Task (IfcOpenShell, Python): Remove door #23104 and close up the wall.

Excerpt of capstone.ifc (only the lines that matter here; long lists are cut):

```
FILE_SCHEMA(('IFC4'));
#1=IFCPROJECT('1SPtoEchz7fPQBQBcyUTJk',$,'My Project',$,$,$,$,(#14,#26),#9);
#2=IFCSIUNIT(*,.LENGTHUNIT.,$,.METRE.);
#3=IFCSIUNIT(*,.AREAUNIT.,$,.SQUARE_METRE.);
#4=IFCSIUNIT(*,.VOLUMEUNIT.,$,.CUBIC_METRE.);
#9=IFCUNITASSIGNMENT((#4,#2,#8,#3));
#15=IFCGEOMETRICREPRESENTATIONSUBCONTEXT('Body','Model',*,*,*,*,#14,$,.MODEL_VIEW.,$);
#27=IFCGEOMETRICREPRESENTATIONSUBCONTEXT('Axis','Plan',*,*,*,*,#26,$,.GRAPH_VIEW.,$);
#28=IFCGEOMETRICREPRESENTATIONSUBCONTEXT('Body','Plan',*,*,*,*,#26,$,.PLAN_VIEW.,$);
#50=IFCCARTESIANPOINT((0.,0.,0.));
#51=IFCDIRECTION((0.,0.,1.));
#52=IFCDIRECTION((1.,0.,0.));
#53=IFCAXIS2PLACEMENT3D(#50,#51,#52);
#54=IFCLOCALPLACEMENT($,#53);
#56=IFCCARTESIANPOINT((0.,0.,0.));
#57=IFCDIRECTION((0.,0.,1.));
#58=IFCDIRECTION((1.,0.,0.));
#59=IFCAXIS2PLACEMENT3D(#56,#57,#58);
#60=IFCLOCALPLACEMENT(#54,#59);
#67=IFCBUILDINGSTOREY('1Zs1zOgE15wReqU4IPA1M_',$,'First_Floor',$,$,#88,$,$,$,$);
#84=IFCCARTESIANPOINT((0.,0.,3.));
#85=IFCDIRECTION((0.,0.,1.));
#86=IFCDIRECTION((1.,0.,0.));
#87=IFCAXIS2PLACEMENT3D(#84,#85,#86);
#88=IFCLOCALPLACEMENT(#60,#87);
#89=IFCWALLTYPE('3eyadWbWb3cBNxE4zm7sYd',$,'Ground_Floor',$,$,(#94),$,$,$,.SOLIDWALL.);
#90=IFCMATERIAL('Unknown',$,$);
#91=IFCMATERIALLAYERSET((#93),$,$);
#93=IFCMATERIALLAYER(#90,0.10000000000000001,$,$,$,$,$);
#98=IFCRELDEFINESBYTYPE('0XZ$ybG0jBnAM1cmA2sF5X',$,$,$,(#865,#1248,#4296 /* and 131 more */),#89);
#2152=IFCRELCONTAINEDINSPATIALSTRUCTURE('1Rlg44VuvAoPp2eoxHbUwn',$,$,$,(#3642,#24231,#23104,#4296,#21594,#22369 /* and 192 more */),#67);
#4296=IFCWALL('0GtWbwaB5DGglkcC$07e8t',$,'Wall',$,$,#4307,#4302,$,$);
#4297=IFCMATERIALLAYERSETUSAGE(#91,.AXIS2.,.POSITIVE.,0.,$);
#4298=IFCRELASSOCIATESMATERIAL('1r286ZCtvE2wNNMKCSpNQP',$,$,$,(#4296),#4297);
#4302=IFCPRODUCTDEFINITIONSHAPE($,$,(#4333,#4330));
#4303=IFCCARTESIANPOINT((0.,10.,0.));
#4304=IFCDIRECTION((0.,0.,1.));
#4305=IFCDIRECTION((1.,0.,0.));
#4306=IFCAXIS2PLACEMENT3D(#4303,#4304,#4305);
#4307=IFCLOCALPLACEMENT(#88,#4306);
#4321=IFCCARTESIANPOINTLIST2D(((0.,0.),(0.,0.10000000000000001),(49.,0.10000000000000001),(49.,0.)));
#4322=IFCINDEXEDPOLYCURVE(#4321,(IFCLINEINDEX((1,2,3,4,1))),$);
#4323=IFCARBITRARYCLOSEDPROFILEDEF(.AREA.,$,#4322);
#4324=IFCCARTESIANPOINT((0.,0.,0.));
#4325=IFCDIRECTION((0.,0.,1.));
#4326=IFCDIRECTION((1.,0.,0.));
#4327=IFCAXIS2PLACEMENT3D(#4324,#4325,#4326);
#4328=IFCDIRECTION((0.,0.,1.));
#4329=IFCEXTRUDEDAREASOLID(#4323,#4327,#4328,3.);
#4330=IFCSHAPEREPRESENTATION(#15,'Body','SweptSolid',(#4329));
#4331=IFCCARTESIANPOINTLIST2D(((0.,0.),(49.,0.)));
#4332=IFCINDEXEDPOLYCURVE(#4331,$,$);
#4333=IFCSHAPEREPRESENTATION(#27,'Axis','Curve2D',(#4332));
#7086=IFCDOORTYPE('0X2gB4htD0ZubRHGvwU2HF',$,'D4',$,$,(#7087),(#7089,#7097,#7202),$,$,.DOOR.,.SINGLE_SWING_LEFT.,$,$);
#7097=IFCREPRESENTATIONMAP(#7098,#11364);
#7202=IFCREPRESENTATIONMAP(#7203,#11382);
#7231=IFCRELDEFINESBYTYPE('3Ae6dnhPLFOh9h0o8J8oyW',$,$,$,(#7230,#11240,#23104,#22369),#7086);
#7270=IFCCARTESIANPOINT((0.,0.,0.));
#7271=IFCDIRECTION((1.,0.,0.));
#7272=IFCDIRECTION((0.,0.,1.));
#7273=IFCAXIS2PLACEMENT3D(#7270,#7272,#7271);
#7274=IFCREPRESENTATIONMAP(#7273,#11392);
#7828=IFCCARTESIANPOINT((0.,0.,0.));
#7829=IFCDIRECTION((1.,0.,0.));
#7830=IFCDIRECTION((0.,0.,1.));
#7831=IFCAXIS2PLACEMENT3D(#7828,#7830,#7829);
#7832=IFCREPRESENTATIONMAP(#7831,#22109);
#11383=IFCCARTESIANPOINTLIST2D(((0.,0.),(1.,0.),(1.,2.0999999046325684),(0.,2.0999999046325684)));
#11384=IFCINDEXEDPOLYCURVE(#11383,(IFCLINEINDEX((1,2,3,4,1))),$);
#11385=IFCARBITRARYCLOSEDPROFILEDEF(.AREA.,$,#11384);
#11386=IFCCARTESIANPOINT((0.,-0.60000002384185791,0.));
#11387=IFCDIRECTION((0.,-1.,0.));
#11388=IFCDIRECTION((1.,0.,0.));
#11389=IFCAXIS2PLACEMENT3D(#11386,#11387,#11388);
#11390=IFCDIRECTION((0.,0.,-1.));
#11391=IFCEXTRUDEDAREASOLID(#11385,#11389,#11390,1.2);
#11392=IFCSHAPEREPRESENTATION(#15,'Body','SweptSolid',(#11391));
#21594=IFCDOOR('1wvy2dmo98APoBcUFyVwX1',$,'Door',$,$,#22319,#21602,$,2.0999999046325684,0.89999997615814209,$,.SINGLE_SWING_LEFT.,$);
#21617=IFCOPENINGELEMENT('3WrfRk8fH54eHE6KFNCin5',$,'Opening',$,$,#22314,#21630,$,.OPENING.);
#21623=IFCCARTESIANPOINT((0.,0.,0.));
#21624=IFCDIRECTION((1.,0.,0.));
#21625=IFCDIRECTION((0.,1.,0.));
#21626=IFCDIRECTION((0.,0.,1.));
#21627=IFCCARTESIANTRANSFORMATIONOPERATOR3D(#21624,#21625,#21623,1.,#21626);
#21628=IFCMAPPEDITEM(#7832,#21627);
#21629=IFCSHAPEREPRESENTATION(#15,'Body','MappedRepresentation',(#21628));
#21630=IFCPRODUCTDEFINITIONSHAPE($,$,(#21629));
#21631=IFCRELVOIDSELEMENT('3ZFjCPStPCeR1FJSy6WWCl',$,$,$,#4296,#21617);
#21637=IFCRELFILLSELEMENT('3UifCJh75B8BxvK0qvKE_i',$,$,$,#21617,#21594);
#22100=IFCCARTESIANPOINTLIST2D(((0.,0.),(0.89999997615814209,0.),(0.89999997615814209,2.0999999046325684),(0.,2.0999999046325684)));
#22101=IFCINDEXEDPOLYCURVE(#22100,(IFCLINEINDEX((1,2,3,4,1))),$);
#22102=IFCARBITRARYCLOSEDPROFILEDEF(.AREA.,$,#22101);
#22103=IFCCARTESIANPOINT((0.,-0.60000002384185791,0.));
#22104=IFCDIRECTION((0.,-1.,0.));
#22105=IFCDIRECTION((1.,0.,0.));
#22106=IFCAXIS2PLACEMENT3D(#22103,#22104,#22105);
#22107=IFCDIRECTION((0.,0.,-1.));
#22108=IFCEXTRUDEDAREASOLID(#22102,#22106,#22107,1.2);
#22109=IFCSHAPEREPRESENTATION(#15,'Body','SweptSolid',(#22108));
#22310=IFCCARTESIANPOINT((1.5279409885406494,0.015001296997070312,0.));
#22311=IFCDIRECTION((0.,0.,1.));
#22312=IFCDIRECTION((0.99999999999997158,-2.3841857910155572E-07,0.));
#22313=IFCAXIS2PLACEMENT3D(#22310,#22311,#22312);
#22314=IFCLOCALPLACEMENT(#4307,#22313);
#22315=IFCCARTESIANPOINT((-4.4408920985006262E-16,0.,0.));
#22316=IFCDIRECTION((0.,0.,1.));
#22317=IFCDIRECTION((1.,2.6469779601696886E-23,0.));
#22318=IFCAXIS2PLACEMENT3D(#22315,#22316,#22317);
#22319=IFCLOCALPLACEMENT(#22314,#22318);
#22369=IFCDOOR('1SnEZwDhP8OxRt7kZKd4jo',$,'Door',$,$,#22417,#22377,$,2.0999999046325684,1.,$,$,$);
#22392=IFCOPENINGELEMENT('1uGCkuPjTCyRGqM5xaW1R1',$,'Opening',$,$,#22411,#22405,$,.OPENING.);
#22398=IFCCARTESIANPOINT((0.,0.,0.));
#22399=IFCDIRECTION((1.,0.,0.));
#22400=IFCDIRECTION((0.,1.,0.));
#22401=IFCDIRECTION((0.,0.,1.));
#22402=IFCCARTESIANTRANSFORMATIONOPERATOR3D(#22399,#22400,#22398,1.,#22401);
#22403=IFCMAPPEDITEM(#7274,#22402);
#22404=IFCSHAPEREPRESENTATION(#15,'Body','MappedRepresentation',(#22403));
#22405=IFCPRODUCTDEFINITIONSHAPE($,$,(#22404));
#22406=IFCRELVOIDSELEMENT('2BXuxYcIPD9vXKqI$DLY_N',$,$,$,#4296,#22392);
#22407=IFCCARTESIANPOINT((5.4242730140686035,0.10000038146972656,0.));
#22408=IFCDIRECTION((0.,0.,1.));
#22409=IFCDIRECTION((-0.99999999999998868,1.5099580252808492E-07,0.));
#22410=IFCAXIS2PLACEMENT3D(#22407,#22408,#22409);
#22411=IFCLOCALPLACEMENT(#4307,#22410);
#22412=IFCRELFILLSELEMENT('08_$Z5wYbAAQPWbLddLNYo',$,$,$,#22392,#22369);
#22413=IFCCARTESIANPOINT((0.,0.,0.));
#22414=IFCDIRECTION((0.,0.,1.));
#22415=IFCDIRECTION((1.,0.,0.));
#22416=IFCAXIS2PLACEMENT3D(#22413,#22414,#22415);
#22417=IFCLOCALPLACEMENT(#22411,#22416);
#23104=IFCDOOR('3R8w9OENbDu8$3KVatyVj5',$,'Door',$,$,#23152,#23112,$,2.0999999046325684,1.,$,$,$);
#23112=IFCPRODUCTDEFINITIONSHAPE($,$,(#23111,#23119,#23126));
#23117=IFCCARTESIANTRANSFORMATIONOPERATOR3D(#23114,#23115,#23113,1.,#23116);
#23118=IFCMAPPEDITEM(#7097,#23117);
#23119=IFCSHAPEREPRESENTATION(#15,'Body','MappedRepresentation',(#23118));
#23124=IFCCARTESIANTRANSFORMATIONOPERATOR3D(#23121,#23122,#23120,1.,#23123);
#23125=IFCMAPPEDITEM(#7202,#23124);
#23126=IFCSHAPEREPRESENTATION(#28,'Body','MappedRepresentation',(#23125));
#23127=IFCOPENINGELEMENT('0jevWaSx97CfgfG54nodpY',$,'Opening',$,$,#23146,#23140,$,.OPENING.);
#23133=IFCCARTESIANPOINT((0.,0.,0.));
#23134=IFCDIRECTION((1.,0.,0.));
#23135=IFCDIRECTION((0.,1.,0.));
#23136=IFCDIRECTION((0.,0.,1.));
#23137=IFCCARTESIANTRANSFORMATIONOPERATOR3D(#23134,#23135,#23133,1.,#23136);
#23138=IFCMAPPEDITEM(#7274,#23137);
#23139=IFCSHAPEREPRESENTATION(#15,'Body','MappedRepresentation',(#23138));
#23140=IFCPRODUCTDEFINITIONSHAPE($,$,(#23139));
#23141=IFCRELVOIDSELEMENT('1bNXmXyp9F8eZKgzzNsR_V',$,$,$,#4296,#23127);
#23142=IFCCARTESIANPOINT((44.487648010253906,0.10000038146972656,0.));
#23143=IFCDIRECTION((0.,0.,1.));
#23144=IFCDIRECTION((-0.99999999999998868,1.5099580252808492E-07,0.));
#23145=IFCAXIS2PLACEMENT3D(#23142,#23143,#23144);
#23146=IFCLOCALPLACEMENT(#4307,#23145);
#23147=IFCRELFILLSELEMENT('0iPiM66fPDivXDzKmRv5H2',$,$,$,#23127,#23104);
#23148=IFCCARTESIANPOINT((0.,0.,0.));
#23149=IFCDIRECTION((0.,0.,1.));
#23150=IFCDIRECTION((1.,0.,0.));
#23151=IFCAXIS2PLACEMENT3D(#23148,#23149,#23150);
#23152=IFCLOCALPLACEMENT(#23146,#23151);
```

```python
import ifcopenshell
import ifcopenshell.api.feature
import ifcopenshell.api.root
import ifcopenshell.geom
import ifcopenshell.util.shape

model = ifcopenshell.open("capstone.ifc")
settings = ifcopenshell.geom.settings()


def volume(element):
    """Net volume in cubic metres, openings subtracted."""
    shape = ifcopenshell.geom.create_shape(settings, element)
    return ifcopenshell.util.shape.get_volume(shape.geometry)


door = model.by_guid("3R8w9OENbDu8$3KVatyVj5")
opening = door.FillsVoids[0].RelatingOpeningElement
wall = opening.VoidsElements[0].RelatingBuildingElement
before = volume(wall)

ifcopenshell.api.root.remove_product(model, product=door)
ifcopenshell.api.feature.remove_feature(model, feature=opening)

after = volume(wall)

print(f"wall volume {before:.3f} -> {after:.3f} m3")

model.write("capstone-out.ifc")
```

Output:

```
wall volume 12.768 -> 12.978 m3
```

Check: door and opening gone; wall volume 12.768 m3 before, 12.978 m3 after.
